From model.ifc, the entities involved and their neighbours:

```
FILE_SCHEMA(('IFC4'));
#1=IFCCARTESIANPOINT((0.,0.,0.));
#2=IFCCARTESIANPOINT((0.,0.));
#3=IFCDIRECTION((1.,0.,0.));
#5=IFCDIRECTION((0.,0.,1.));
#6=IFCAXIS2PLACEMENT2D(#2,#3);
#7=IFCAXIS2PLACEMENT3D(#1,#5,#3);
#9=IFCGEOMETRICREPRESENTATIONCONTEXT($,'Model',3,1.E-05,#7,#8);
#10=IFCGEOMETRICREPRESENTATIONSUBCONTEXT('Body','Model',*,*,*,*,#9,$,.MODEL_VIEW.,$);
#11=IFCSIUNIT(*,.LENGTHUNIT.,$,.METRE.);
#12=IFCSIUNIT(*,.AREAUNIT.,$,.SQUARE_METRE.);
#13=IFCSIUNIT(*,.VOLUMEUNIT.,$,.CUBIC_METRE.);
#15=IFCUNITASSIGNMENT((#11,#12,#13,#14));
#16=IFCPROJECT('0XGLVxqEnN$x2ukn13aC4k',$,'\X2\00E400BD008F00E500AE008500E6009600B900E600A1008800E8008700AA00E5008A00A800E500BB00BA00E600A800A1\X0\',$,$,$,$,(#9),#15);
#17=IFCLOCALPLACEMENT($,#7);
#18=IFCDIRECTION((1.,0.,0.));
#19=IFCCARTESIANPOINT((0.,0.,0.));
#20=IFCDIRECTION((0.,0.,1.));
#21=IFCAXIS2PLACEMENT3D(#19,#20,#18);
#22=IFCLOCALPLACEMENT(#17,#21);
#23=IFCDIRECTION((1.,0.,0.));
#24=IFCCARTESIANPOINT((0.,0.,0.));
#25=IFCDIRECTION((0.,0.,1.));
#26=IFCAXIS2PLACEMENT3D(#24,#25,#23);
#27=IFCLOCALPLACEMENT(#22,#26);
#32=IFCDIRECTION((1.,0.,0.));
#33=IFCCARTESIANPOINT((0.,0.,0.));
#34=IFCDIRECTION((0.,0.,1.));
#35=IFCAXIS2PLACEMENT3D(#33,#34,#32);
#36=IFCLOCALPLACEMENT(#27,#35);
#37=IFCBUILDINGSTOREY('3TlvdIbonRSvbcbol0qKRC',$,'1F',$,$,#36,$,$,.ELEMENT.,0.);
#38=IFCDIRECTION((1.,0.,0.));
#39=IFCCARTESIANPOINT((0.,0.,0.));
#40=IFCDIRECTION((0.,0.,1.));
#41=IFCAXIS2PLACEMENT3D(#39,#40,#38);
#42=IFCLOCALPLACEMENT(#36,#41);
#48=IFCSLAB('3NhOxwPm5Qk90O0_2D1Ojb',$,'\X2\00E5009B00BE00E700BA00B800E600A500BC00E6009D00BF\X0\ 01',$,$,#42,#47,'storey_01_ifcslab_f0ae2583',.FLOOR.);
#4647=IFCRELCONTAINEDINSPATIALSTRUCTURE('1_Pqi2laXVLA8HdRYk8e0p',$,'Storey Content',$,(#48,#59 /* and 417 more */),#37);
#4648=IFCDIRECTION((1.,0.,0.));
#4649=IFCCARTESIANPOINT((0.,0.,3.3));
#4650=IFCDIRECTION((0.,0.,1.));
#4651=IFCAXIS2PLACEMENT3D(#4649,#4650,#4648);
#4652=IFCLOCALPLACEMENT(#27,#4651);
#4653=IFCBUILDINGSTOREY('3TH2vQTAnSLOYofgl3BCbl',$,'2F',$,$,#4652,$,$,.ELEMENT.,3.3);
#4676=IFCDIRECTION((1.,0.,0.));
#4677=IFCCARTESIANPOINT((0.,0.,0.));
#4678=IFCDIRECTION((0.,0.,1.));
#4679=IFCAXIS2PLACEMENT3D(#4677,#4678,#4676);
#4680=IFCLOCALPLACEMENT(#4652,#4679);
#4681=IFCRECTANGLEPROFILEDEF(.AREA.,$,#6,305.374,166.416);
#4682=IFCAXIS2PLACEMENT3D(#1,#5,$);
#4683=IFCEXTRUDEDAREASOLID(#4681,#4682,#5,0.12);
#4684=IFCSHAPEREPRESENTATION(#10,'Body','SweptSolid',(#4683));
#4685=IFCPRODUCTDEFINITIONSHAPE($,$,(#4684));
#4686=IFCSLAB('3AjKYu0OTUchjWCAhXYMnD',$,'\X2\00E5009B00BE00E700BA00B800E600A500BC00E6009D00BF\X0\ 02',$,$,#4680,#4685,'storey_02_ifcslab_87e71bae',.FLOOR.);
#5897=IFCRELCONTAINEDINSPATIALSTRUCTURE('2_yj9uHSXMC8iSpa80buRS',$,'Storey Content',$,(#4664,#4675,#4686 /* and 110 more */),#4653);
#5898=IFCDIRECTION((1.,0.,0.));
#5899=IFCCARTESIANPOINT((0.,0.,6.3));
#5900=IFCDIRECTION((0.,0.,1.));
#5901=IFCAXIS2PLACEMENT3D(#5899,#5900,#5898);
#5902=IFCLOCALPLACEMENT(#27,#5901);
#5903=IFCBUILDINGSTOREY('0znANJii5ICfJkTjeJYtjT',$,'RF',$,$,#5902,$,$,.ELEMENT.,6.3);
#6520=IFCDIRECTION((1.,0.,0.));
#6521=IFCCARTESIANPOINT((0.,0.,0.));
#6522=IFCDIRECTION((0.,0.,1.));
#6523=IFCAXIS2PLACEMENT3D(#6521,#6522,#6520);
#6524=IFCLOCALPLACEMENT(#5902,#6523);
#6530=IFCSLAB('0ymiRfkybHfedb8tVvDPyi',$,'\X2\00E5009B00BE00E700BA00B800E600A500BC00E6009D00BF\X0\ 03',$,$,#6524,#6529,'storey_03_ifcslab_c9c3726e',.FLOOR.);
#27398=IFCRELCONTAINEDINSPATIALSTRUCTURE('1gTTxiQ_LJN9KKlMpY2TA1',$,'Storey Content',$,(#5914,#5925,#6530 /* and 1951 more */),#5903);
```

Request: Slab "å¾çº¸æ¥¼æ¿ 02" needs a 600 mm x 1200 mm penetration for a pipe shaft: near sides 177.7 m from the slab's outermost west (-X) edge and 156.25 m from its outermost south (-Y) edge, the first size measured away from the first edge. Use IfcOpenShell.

```python
import numpy as np
import ifcopenshell
import ifcopenshell.api.feature
import ifcopenshell.api.geometry
import ifcopenshell.api.root
import ifcopenshell.geom
import ifcopenshell.util.placement
import ifcopenshell.util.representation
import ifcopenshell.util.shape
import ifcopenshell.util.unit

model = ifcopenshell.open("model.ifc")
unit_scale = ifcopenshell.util.unit.calculate_unit_scale(model)
settings = ifcopenshell.geom.settings()


def volume(element):
    """Net volume in cubic metres, openings subtracted."""
    shape = ifcopenshell.geom.create_shape(settings, element)
    return ifcopenshell.util.shape.get_volume(shape.geometry)


slab = model.by_guid("3AjKYu0OTUchjWCAhXYMnD")
before = volume(slab)

# Extent in the slab's own axes, in metres. The edges named are its -X and -Y sides.
slab_shape = ifcopenshell.geom.create_shape(settings, slab)
vertices = ifcopenshell.util.shape.get_vertices(slab_shape.geometry)
x_min, y_min, bottom = vertices.min(axis=0)
top = vertices[:, 2].max()

opening = ifcopenshell.api.root.create_entity(model, ifc_class="IfcOpeningElement", name="Pipe shaft opening", predefined_type="OPENING")
context = ifcopenshell.util.representation.get_context(model, "Model", "Body", "MODEL_VIEW")
width, depth = 0.6, 1.2
outline = [(0.0, 0.0), (width, 0.0), (width, depth), (0.0, depth), (0.0, 0.0)]
# Overshoot both faces by 50 mm so the cut is clean.
shape = ifcopenshell.api.geometry.add_slab_representation(
    model, context=context, depth=top - bottom + 0.1, polyline=outline
)
ifcopenshell.api.geometry.assign_representation(model, product=opening, representation=shape)

matrix = ifcopenshell.util.placement.get_local_placement(slab.ObjectPlacement)
matrix[:, 3] = matrix @ np.append(np.array([x_min + 177.7, y_min + 156.25, bottom - 0.05]) / unit_scale, 1.0)
ifcopenshell.api.geometry.edit_object_placement(model, product=opening, matrix=matrix, is_si=False)
ifcopenshell.api.feature.add_feature(model, feature=opening, element=slab)

after = volume(slab)

print(f"slab volume {before:.3f} -> {after:.3f} m3")

model.write("model_updated.ifc")
```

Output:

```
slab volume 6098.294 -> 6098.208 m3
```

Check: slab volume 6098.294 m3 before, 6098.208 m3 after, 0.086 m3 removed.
